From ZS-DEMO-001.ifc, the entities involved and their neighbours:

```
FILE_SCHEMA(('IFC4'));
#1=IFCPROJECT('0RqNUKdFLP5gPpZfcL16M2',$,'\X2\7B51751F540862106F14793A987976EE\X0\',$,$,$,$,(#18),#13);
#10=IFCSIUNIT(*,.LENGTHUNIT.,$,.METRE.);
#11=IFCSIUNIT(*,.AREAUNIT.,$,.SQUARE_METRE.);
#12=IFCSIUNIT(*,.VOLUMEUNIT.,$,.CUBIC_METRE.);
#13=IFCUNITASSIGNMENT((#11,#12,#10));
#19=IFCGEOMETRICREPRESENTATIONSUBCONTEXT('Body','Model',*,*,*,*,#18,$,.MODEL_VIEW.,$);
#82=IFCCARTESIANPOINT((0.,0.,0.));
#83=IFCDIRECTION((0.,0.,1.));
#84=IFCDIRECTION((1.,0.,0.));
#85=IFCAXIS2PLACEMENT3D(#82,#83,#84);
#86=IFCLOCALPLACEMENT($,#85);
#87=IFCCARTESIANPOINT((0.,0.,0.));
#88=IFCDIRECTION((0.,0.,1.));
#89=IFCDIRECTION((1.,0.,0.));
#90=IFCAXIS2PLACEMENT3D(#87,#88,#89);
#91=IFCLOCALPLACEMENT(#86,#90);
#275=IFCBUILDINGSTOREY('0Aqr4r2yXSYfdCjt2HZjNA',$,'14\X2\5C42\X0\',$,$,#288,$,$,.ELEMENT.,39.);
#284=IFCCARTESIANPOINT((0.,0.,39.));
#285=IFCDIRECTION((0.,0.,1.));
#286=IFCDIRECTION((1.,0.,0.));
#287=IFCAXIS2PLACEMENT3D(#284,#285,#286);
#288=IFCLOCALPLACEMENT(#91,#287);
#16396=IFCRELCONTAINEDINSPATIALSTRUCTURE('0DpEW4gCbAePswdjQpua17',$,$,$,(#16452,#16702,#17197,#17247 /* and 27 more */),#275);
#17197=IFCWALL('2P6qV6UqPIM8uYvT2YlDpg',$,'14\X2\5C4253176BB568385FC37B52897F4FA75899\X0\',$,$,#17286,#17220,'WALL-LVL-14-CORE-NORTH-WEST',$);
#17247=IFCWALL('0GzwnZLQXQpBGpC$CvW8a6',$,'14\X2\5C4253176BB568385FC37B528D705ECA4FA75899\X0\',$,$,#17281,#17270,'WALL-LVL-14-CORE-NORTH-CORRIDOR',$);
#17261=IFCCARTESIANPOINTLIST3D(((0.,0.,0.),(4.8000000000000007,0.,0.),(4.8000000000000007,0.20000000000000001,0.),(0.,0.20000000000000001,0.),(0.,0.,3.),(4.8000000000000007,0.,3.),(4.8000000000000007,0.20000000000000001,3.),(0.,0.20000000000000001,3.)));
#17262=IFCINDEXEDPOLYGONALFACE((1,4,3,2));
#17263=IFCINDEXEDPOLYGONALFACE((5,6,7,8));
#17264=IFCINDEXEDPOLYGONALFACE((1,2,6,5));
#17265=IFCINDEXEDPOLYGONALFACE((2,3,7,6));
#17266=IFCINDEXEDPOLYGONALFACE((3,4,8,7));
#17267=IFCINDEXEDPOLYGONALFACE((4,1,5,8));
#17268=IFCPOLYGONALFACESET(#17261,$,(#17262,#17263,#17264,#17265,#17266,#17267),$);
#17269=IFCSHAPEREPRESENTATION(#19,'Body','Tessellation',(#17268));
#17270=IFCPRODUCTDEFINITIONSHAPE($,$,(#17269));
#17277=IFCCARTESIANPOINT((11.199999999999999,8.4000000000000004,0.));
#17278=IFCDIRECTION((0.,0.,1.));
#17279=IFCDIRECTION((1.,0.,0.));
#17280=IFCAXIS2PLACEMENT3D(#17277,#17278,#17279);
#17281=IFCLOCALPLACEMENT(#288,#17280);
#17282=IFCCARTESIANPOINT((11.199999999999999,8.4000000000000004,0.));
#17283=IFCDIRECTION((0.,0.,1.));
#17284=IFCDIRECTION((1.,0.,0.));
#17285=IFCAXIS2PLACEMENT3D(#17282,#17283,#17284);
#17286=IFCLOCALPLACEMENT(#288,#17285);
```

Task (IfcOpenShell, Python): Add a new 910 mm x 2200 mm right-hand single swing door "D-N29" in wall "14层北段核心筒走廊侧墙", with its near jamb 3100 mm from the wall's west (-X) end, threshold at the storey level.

```python
import numpy as np
import ifcopenshell
import ifcopenshell.api.feature
import ifcopenshell.api.geometry
import ifcopenshell.api.root
import ifcopenshell.api.spatial
import ifcopenshell.geom
import ifcopenshell.util.element
import ifcopenshell.util.placement
import ifcopenshell.util.representation
import ifcopenshell.util.shape
import ifcopenshell.util.unit

model = ifcopenshell.open("ZS-DEMO-001.ifc")
unit_scale = ifcopenshell.util.unit.calculate_unit_scale(model)
settings = ifcopenshell.geom.settings()


def volume(element):
    """Net volume in cubic metres, openings subtracted."""
    shape = ifcopenshell.geom.create_shape(settings, element)
    return ifcopenshell.util.shape.get_volume(shape.geometry)


wall = model.by_guid("0GzwnZLQXQpBGpC$CvW8a6")
storey = ifcopenshell.util.element.get_container(wall, ifc_class="IfcBuildingStorey")
context = ifcopenshell.util.representation.get_context(model, "Model", "Body", "MODEL_VIEW")
before = volume(wall)

width, height, from_end, sill = 0.91, 2.2, 3.1, 0.0  # metres

# The wall runs along its own X axis, and the end named is its -X end.
wall_shape = ifcopenshell.geom.create_shape(settings, wall)
x, y, z = ifcopenshell.util.shape.get_vertices(wall_shape.geometry).T
start = x.min() + from_end
face, thickness = float(y.min()), float(y.max() - y.min())
wall_matrix = ifcopenshell.util.placement.get_local_placement(wall.ObjectPlacement)
level = ifcopenshell.util.placement.get_local_placement(storey.ObjectPlacement)[2, 3]


def in_wall(x, y):
    """Placement at x, y metres in the wall's axes, at sill height."""
    matrix = wall_matrix.copy()
    matrix[:, 3] = wall_matrix @ np.array([x / unit_scale, y / unit_scale, 0.0, 1.0])
    matrix[2, 3] = level + sill / unit_scale
    return matrix


# Opening: a box that overshoots both wall faces by 50 mm.
opening = ifcopenshell.api.root.create_entity(model, ifc_class="IfcOpeningElement", predefined_type="OPENING")
box = ifcopenshell.api.geometry.add_wall_representation(
    model, context=context, length=width, height=height, thickness=thickness + 0.1
)
ifcopenshell.api.geometry.assign_representation(model, product=opening, representation=box)
ifcopenshell.api.geometry.edit_object_placement(model, product=opening, matrix=in_wall(start, face - 0.05), is_si=False)
ifcopenshell.api.feature.add_feature(model, feature=opening, element=wall)

door = ifcopenshell.api.root.create_entity(model, ifc_class="IfcDoor", name="D-N29", predefined_type="DOOR")
door.OverallWidth, door.OverallHeight = width / unit_scale, height / unit_scale
door.OperationType = "SINGLE_SWING_RIGHT"
body = ifcopenshell.api.geometry.add_door_representation(
    model,
    context=context,
    overall_width=door.OverallWidth,
    overall_height=door.OverallHeight,
    operation_type="SINGLE_SWING_RIGHT",
    lining_properties={"LiningDepth": thickness / unit_scale, "ThresholdDepth": thickness / unit_scale},
)
ifcopenshell.api.geometry.assign_representation(model, product=door, representation=body)
ifcopenshell.api.spatial.assign_container(model, products=[door], relating_structure=storey)
ifcopenshell.api.feature.add_filling(model, opening=opening, element=door)

# The lining spans the wall, so the door starts at the wall face.
ifcopenshell.api.geometry.edit_object_placement(model, product=door, matrix=in_wall(start, face), is_si=False)

after = volume(wall)

print(f"wall volume {before:.3f} -> {after:.3f} m3")

model.write("ZS-DEMO-001-out.ifc")
```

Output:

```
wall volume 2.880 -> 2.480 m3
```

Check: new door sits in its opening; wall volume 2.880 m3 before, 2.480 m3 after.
